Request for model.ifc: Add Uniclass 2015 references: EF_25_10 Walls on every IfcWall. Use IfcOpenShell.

First a look at what the model holds.

```python
import ifcopenshell

model = ifcopenshell.open("model.ifc")
print(model.schema)
print("classifications:", [c.Name for c in model.by_type("IfcClassification")])
for ifc_class in ("IfcDoor", "IfcRoof", "IfcStair", "IfcWall", "IfcWindow"):
    print(ifc_class, len(model.by_type(ifc_class)))
```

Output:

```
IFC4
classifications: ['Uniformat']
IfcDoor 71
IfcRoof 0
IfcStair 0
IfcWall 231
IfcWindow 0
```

```python
import ifcopenshell
import ifcopenshell.api.classification

model = ifcopenshell.open("model.ifc")

system = ifcopenshell.api.classification.add_classification(model, classification="Uniclass 2015")

codes = {
    "IfcWall": ("EF_25_10", "Walls"),
}
for ifc_class, (code, name) in codes.items():
    products = model.by_type(ifc_class)
    ifcopenshell.api.classification.add_reference(
        model, products=products, classification=system, identification=code, name=name
    )
    print(code, len(products))

model.write("model_v2.ifc")
```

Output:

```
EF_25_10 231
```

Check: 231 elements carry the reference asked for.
